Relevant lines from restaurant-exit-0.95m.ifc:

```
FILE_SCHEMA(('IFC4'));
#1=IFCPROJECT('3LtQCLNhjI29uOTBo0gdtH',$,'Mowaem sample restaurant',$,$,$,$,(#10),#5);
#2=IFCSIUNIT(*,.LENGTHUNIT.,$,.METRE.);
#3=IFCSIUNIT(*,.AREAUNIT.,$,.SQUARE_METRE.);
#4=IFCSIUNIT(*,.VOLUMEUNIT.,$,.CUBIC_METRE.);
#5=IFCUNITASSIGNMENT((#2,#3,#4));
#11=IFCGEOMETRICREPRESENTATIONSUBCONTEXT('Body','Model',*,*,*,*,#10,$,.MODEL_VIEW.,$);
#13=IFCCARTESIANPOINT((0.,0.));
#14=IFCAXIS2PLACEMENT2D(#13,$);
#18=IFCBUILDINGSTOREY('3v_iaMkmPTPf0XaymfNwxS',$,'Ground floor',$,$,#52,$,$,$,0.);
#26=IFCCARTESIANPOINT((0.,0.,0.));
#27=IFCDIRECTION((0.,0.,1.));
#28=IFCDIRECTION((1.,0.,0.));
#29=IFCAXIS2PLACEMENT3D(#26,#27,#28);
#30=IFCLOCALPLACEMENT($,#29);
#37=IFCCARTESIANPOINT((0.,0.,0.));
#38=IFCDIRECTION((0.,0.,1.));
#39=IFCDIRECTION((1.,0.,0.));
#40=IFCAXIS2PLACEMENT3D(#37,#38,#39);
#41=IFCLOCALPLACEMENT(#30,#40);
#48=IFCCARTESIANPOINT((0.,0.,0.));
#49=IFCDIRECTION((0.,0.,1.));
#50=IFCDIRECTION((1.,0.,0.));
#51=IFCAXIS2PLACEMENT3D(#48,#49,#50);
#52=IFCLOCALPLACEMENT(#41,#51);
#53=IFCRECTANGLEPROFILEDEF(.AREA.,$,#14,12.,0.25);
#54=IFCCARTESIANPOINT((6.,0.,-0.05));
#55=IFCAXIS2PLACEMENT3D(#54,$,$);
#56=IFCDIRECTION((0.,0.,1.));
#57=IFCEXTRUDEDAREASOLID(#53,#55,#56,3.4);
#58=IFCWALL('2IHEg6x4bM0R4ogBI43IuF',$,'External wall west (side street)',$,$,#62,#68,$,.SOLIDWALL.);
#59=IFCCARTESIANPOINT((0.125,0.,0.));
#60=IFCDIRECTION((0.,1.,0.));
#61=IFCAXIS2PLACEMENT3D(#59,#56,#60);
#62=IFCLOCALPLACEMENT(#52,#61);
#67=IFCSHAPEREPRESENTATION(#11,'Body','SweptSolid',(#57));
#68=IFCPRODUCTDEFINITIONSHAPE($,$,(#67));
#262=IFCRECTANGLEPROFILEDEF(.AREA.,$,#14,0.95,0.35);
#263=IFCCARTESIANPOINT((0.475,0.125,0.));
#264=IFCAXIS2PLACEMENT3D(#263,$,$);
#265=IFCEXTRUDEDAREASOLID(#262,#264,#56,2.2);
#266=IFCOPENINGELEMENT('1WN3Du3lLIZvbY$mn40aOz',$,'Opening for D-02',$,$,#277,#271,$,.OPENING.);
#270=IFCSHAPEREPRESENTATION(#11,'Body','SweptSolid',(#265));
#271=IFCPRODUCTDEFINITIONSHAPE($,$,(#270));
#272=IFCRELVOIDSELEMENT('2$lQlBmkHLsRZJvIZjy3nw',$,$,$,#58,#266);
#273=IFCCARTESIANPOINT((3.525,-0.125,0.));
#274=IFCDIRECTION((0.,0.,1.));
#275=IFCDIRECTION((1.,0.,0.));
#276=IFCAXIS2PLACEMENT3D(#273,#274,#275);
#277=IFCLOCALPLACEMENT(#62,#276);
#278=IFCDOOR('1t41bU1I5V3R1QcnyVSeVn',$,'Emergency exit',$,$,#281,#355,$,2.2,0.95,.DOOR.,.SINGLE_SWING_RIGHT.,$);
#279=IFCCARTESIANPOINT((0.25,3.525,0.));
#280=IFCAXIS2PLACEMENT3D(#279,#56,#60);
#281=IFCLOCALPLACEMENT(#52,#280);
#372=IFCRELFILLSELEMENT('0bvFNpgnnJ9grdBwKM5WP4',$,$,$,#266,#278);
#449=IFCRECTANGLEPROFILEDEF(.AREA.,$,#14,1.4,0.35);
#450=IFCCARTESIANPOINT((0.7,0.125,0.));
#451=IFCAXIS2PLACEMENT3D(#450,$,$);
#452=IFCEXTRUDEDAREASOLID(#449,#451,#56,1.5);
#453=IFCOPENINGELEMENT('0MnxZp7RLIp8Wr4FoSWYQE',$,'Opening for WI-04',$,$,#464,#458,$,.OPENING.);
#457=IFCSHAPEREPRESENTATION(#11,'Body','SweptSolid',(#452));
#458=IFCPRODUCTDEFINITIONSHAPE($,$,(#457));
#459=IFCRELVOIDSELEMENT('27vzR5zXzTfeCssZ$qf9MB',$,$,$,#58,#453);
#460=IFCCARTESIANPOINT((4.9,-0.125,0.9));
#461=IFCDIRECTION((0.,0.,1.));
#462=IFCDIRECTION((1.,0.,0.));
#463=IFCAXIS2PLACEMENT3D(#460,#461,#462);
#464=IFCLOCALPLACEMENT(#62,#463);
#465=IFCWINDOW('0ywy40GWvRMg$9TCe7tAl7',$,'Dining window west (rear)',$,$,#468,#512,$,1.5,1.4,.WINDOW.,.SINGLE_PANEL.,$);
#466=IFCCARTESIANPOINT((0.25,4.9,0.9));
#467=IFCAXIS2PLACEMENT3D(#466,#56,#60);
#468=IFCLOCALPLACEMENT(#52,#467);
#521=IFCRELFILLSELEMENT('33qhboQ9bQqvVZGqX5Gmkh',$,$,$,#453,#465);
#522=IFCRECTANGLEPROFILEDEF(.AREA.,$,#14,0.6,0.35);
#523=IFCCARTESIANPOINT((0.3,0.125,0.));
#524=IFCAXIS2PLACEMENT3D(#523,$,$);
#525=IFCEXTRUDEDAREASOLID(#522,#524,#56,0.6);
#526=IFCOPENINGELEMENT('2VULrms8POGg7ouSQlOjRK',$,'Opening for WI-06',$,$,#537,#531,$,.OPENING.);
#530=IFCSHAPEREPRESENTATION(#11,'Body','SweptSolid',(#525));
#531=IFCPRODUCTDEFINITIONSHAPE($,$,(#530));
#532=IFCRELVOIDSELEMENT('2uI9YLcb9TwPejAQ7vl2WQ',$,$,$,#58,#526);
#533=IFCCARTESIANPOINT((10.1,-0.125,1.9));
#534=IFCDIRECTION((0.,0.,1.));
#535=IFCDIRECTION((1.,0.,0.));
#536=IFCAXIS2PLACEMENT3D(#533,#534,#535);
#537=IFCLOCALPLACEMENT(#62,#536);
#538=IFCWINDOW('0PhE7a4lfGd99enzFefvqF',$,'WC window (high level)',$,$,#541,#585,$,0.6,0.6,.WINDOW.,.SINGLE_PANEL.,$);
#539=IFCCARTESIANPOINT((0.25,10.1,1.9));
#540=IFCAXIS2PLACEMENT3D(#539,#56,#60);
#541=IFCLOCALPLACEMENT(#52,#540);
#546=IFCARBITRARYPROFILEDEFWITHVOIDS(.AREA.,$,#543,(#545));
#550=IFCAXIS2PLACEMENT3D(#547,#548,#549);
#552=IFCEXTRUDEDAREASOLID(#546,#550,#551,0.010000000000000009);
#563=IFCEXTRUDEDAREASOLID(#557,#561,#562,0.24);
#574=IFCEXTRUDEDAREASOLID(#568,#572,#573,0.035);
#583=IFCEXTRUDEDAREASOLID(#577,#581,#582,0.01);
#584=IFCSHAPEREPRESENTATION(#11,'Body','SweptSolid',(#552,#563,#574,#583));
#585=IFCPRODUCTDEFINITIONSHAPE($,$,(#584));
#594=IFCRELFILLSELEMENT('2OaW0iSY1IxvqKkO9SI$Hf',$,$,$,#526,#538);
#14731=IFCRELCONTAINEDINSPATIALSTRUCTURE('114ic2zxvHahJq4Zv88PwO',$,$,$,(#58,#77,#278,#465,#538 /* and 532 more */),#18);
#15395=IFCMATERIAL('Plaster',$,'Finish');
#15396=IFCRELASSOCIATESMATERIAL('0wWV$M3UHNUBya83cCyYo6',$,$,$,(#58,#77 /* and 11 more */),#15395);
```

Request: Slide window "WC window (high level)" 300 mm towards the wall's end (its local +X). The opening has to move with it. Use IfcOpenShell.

```python
import ifcopenshell
import ifcopenshell.api.geometry
import ifcopenshell.util.placement
import ifcopenshell.util.unit

model = ifcopenshell.open("restaurant-exit-0.95m.ifc")
unit_scale = ifcopenshell.util.unit.calculate_unit_scale(model)

window = model.by_id(538)
opening = window.FillsVoids[0].RelatingOpeningElement
wall = opening.VoidsElements[0].RelatingBuildingElement

wall_matrix = ifcopenshell.util.placement.get_local_placement(wall.ObjectPlacement)
shift = wall_matrix[:3, 0] * 0.3 / unit_scale
before = ifcopenshell.util.placement.get_local_placement(window.ObjectPlacement)[:3, 3].copy()

# The window is not placed relative to its opening, so move both.
for product in (opening, window):
    matrix = ifcopenshell.util.placement.get_local_placement(product.ObjectPlacement)
    matrix[:3, 3] += shift
    ifcopenshell.api.geometry.edit_object_placement(model, product=product, matrix=matrix, is_si=False)

after = ifcopenshell.util.placement.get_local_placement(window.ObjectPlacement)[:3, 3]
print("window moved by", (after - before).round(3) + 0.0)

model.write("restaurant-exit-0.95m_rev.ifc")
```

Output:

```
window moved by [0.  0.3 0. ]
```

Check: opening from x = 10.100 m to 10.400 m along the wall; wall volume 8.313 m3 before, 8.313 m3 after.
